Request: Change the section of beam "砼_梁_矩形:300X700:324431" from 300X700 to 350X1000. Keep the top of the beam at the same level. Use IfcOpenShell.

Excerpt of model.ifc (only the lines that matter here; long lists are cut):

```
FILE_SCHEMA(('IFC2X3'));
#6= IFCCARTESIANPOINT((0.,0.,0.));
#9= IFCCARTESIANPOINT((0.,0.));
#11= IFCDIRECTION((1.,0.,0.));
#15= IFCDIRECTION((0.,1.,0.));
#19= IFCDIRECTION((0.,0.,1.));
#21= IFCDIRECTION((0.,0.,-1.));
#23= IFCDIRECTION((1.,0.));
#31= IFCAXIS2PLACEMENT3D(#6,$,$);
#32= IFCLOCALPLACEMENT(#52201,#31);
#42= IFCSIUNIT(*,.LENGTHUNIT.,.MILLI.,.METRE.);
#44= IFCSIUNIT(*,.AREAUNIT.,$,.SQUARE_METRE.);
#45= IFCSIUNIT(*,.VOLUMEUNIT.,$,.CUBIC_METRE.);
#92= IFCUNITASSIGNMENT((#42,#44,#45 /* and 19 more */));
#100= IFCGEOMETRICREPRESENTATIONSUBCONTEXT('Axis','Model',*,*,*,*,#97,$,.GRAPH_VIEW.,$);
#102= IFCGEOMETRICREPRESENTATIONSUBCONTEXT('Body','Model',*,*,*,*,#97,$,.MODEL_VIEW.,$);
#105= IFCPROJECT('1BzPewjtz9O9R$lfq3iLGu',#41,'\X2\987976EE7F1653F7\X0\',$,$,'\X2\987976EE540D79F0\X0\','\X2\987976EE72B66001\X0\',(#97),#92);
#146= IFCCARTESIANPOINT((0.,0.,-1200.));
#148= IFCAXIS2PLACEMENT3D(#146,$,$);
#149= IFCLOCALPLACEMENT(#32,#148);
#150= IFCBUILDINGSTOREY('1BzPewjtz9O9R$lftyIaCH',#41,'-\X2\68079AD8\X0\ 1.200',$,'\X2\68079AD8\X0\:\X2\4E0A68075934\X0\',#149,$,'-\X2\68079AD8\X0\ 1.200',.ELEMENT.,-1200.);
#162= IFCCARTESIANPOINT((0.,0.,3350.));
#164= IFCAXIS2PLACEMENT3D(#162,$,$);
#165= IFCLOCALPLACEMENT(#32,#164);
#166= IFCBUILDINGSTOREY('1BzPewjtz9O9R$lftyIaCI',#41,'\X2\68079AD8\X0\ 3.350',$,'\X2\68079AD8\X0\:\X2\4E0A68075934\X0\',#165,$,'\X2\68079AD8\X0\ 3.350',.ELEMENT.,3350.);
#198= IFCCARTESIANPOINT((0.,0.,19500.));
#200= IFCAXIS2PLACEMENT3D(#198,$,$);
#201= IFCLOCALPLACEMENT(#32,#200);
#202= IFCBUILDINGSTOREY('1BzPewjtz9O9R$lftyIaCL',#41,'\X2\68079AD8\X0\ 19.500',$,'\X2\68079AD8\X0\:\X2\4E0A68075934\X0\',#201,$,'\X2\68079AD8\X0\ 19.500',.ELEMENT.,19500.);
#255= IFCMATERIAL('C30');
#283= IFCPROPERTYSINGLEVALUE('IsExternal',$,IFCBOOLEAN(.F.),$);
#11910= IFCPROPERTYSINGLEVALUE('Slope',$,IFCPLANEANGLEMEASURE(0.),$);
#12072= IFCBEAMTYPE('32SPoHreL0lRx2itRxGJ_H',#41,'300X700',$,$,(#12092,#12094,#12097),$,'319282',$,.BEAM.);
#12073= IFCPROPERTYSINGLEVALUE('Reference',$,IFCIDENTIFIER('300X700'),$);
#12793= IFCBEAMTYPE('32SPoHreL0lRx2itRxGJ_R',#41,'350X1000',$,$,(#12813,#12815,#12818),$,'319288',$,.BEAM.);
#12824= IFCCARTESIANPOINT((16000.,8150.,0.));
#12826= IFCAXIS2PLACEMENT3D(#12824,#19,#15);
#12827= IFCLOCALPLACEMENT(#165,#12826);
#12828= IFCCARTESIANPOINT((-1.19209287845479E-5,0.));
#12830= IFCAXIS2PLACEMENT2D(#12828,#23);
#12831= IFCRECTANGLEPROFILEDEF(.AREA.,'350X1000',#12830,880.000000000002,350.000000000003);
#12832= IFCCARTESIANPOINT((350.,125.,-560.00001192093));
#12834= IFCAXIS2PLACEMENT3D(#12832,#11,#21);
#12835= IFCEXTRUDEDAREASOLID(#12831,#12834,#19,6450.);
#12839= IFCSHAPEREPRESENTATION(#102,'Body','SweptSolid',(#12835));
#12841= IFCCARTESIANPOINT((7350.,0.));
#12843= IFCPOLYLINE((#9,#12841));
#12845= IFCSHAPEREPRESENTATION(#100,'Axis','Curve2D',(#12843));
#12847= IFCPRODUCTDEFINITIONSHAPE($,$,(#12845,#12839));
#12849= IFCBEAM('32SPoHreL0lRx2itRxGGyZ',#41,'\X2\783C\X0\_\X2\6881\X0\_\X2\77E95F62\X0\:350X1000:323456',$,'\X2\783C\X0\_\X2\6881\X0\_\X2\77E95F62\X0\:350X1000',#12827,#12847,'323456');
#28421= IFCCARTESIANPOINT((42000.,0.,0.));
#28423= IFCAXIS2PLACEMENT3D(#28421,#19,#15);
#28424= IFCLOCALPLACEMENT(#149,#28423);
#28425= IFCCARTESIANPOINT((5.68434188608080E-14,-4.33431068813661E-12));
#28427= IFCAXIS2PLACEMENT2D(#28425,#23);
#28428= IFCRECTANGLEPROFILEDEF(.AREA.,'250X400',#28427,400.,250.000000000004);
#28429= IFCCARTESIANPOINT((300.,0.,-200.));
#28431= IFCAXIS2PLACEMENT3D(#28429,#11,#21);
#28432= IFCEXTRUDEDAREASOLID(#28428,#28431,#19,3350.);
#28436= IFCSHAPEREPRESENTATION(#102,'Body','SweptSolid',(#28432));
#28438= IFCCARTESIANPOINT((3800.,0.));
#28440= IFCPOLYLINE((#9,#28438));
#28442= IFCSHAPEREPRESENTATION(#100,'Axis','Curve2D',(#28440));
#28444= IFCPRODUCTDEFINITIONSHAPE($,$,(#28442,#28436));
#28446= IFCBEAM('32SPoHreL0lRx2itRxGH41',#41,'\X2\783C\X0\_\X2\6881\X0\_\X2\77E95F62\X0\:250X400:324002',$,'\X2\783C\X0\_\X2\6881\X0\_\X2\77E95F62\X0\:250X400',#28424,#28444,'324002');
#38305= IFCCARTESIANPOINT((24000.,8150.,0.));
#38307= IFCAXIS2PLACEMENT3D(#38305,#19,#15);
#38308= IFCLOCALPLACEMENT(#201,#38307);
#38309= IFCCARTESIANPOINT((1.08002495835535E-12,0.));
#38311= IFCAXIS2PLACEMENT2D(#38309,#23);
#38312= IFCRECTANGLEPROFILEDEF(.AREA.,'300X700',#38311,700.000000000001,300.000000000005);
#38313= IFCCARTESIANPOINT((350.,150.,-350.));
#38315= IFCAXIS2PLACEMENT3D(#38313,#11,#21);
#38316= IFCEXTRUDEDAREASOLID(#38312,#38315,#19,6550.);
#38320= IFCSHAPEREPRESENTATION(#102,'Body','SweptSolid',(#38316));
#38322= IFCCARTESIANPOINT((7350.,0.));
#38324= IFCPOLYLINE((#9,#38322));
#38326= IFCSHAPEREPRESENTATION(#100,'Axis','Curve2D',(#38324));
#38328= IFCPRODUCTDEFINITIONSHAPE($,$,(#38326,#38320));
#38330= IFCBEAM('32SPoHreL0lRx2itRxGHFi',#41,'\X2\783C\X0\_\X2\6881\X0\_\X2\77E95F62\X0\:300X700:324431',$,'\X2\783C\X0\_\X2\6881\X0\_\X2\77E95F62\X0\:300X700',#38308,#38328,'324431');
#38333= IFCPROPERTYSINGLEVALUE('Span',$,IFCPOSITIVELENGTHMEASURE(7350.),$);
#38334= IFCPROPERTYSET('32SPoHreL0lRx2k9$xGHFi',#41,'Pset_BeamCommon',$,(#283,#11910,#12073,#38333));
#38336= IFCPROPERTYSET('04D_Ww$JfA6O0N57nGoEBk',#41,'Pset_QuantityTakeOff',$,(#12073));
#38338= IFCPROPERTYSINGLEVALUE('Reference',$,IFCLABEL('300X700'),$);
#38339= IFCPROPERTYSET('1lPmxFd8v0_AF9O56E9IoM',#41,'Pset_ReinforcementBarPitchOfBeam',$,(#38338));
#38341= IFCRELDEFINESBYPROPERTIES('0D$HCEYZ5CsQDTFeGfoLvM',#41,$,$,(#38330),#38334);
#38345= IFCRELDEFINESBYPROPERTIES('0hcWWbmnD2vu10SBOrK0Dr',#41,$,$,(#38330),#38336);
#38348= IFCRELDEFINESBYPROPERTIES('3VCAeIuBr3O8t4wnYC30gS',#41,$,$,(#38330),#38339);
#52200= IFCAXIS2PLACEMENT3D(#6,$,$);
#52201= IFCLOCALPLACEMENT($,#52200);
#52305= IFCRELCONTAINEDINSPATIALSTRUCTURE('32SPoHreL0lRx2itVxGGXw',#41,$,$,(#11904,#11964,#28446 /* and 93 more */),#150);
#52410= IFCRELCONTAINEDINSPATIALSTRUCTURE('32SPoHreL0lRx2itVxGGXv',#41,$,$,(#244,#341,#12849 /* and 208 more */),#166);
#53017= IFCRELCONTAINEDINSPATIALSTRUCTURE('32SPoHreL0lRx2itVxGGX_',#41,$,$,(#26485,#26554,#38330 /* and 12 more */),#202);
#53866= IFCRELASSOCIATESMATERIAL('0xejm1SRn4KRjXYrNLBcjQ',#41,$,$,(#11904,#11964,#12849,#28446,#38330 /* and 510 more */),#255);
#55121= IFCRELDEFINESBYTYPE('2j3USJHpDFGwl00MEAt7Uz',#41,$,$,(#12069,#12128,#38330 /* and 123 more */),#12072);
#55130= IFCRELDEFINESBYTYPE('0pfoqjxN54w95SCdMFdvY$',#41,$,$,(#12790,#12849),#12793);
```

```python
import ifcopenshell
import ifcopenshell.api.pset
import ifcopenshell.api.type
import ifcopenshell.util.element
import ifcopenshell.util.representation

model = ifcopenshell.open("model.ifc")

member = model.by_id(38330)
source = next(p for p in model.by_type("IfcRectangleProfileDef") if p.ProfileName == "350X1000")

body = ifcopenshell.util.representation.get_representation(member, "Model", "Body")
solid = body.Items[0]
old_profile = solid.SweptArea

# Copy the section's sizes but keep this member's own profile position.
profile = ifcopenshell.util.element.copy(model, source)
# Profiles are centred, so shift by half the change in depth to hold the top.
shift = (old_profile.XDim - profile.XDim) / 2
x, y = old_profile.Position.Location.Coordinates
up = (-1.0, 0.0)  # upwards, in the solid's own plane
location = model.createIfcCartesianPoint((x + up[0] * shift, y + up[1] * shift))
profile.Position = model.createIfcAxis2Placement2D(location, old_profile.Position.RefDirection)
solid.SweptArea = profile
if not model.get_total_inverses(old_profile):
    ifcopenshell.util.element.remove_deep2(model, old_profile)

new_type = model.by_id(12793)
ifcopenshell.api.type.assign_type(
    model, related_objects=[member], relating_type=new_type, should_map_representations=False
)
member.Name = member.Name.replace("300X700", "350X1000")
member.ObjectType = "砼_梁_矩形:350X1000"
pset = model.by_id(ifcopenshell.util.element.get_pset(member, "Pset_BeamCommon", should_inherit=False)["id"])
ifcopenshell.api.pset.edit_pset(model, pset=pset, properties={"Reference": "350X1000"})
pset = model.by_id(ifcopenshell.util.element.get_pset(member, "Pset_QuantityTakeOff", should_inherit=False)["id"])
ifcopenshell.api.pset.edit_pset(model, pset=pset, properties={"Reference": "350X1000"})
pset = model.by_id(ifcopenshell.util.element.get_pset(member, "Pset_ReinforcementBarPitchOfBeam", should_inherit=False)["id"])
ifcopenshell.api.pset.edit_pset(model, pset=pset, properties={"Reference": "350X1000"})

print(solid.SweptArea)

model.write("model-out.ifc")
```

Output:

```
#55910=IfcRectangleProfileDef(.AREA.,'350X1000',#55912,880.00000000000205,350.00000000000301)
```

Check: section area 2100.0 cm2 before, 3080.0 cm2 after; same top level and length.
